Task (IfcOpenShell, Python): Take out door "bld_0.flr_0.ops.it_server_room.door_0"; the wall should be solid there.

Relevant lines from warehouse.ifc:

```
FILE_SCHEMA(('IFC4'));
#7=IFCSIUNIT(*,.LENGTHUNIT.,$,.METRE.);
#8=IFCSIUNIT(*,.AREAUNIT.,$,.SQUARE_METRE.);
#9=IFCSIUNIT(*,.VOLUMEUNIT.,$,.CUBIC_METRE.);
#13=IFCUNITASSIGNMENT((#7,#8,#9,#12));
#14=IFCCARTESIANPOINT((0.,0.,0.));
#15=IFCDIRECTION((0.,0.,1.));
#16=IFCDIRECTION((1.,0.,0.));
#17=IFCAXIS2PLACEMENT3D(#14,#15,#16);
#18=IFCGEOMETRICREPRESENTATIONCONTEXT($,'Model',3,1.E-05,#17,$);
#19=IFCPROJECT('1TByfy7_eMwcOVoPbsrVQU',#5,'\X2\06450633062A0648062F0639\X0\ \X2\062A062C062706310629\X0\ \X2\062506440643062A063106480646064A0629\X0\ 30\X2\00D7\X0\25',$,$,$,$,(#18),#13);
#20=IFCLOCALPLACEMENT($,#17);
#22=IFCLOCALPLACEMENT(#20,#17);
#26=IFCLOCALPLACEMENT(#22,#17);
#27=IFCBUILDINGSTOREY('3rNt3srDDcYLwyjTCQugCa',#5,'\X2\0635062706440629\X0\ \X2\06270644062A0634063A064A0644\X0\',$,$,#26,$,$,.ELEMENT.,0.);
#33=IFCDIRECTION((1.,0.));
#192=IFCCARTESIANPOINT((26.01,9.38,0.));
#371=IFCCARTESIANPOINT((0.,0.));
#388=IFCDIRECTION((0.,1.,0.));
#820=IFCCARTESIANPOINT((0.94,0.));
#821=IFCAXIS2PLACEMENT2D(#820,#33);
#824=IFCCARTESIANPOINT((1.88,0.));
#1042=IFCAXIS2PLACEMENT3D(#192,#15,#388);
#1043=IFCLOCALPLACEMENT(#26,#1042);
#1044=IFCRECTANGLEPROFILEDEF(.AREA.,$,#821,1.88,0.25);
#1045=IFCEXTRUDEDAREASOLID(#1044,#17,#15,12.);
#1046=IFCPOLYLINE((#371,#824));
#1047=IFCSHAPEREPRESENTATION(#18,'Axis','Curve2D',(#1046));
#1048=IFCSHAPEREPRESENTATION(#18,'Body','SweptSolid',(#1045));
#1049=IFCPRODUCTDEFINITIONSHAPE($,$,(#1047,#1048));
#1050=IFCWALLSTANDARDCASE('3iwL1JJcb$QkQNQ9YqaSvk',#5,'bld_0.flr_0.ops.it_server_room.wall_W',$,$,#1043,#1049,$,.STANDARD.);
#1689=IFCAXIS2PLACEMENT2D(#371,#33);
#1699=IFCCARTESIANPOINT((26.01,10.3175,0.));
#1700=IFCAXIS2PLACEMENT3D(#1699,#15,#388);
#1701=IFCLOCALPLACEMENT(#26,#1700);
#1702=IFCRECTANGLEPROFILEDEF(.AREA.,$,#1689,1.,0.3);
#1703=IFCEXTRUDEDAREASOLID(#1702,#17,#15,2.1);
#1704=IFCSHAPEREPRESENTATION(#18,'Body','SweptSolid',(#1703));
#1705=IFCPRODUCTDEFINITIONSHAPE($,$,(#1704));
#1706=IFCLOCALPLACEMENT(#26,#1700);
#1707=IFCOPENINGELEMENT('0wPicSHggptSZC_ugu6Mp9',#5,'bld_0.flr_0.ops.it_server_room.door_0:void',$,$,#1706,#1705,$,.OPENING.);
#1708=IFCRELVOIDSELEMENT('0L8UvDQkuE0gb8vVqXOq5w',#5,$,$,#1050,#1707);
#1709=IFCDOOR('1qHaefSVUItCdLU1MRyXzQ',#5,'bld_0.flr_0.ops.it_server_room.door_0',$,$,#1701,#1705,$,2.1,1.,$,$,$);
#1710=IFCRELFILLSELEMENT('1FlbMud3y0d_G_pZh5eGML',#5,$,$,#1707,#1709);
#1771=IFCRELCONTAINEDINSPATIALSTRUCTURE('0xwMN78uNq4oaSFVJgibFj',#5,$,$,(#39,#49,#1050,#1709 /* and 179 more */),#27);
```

```python
import ifcopenshell
import ifcopenshell.api.feature
import ifcopenshell.api.root
import ifcopenshell.geom
import ifcopenshell.util.shape

model = ifcopenshell.open("warehouse.ifc")
settings = ifcopenshell.geom.settings()


def volume(element):
    """Net volume in cubic metres, openings subtracted."""
    shape = ifcopenshell.geom.create_shape(settings, element)
    return ifcopenshell.util.shape.get_volume(shape.geometry)


door = model.by_id(1709)
opening = door.FillsVoids[0].RelatingOpeningElement
wall = opening.VoidsElements[0].RelatingBuildingElement
before = volume(wall)

ifcopenshell.api.root.remove_product(model, product=door)
ifcopenshell.api.feature.remove_feature(model, feature=opening)

after = volume(wall)

print(f"wall volume {before:.3f} -> {after:.3f} m3")

model.write("warehouse_v2.ifc")
```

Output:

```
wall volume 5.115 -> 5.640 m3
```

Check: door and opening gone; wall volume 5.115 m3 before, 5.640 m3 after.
